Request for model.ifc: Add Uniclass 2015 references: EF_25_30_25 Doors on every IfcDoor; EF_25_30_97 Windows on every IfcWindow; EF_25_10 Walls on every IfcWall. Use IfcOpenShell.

First a look at what the model holds.

```python
import ifcopenshell

model = ifcopenshell.open("model.ifc")
print(model.schema)
print("classifications:", [c.Name for c in model.by_type("IfcClassification")])
for ifc_class in ("IfcDoor", "IfcRoof", "IfcStair", "IfcWall", "IfcWindow"):
    print(ifc_class, len(model.by_type(ifc_class)))
```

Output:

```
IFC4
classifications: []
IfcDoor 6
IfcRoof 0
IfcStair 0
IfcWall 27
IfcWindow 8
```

```python
import ifcopenshell
import ifcopenshell.api.classification

model = ifcopenshell.open("model.ifc")

system = ifcopenshell.api.classification.add_classification(model, classification="Uniclass 2015")

codes = {
    "IfcDoor": ("EF_25_30_25", "Doors"),
    "IfcWindow": ("EF_25_30_97", "Windows"),
    "IfcWall": ("EF_25_10", "Walls"),
}
for ifc_class, (code, name) in codes.items():
    products = model.by_type(ifc_class)
    ifcopenshell.api.classification.add_reference(
        model, products=products, classification=system, identification=code, name=name
    )
    print(code, len(products))

model.write("model_v2.ifc")
```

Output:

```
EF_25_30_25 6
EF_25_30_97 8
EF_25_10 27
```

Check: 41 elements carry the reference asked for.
